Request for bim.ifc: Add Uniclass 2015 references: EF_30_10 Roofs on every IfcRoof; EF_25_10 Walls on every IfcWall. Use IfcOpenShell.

First a look at what the model holds.

```python
import ifcopenshell

model = ifcopenshell.open("bim.ifc")
print(model.schema)
print("classifications:", [c.Name for c in model.by_type("IfcClassification")])
for ifc_class in ("IfcDoor", "IfcRoof", "IfcStair", "IfcWall", "IfcWindow"):
    print(ifc_class, len(model.by_type(ifc_class)))
```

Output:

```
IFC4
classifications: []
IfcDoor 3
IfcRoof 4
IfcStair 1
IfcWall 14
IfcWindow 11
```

```python
import ifcopenshell
import ifcopenshell.api.classification

model = ifcopenshell.open("bim.ifc")

system = ifcopenshell.api.classification.add_classification(model, classification="Uniclass 2015")

codes = {
    "IfcRoof": ("EF_30_10", "Roofs"),
    "IfcWall": ("EF_25_10", "Walls"),
}
for ifc_class, (code, name) in codes.items():
    products = model.by_type(ifc_class)
    ifcopenshell.api.classification.add_reference(
        model, products=products, classification=system, identification=code, name=name
    )
    print(code, len(products))

model.write("bim-out.ifc")
```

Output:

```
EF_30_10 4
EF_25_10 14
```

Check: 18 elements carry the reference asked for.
